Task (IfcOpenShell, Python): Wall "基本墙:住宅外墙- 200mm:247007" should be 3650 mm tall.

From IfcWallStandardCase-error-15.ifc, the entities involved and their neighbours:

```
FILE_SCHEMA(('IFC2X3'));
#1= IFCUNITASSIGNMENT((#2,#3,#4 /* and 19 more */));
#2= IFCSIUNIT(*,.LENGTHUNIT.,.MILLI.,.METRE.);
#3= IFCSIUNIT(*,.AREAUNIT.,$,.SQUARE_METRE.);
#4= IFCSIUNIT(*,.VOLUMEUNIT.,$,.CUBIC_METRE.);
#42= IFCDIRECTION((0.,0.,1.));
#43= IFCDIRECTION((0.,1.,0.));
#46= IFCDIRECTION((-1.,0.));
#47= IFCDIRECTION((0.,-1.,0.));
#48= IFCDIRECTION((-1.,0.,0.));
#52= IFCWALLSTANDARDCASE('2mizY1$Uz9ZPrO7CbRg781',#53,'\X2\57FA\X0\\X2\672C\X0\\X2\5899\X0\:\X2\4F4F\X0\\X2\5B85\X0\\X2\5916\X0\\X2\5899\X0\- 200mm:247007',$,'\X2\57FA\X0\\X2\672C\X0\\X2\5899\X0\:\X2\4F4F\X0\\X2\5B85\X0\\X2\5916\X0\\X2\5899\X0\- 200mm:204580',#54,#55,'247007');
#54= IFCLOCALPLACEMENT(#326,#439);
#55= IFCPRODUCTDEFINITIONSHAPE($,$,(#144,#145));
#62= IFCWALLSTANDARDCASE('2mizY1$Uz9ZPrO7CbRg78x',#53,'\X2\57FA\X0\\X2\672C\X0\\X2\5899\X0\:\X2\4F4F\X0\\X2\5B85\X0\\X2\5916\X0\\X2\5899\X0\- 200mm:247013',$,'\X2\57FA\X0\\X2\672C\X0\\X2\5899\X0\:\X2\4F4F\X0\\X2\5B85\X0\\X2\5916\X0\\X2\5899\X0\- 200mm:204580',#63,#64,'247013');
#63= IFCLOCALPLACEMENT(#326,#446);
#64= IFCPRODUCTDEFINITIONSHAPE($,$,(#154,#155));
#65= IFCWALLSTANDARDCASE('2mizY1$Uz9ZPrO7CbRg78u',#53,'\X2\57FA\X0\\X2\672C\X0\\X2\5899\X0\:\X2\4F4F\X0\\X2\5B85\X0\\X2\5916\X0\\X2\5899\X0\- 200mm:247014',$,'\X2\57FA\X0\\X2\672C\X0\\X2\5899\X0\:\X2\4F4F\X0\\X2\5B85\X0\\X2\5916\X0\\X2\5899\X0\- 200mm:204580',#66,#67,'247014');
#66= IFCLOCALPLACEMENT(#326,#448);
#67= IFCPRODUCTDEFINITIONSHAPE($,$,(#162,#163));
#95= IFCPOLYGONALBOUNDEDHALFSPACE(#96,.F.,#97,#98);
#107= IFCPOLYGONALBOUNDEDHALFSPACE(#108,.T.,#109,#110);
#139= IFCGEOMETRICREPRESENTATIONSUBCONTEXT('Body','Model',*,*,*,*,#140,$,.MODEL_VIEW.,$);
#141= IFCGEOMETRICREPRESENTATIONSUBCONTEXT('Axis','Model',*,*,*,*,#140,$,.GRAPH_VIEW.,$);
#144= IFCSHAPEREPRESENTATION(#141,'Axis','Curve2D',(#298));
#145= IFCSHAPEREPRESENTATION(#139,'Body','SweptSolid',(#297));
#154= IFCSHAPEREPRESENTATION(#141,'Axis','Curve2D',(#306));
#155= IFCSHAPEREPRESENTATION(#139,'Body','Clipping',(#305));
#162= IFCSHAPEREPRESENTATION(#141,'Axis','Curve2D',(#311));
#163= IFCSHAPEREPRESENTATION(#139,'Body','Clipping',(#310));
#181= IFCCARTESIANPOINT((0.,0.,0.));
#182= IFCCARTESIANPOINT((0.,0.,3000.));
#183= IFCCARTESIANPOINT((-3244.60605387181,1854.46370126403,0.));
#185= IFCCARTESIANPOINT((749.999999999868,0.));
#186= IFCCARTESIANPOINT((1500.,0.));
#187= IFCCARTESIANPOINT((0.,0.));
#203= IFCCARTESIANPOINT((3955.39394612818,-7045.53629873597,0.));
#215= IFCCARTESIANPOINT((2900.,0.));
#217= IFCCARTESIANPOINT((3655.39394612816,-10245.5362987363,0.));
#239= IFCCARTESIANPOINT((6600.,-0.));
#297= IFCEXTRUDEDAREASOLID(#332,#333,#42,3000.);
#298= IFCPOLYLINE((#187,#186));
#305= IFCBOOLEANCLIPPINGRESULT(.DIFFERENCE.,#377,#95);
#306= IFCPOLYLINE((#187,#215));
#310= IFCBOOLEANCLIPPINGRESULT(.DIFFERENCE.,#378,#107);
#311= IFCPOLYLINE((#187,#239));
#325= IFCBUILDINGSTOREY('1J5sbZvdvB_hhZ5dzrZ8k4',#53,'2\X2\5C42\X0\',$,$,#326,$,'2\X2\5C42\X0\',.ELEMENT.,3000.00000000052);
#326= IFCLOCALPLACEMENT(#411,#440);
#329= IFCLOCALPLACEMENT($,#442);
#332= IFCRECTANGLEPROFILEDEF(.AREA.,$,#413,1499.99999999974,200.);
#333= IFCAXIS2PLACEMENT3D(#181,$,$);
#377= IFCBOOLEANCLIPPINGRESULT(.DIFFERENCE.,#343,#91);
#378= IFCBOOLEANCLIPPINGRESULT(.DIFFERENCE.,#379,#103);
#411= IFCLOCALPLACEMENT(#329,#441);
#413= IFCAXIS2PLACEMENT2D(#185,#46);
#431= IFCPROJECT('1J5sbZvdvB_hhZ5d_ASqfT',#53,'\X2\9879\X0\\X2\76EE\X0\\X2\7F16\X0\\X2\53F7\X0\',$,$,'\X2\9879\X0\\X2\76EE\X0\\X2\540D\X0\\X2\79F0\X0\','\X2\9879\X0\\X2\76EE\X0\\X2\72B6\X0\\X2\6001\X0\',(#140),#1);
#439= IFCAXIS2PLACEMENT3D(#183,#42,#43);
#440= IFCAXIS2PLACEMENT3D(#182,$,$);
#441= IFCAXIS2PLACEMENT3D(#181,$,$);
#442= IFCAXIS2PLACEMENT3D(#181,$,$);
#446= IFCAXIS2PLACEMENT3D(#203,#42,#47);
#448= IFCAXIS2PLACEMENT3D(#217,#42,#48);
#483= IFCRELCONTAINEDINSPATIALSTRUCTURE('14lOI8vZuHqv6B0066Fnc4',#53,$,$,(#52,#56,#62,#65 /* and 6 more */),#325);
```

```python
import ifcopenshell
import ifcopenshell.geom
import ifcopenshell.util.representation
import ifcopenshell.util.shape

model = ifcopenshell.open("IfcWallStandardCase-error-15.ifc")
settings = ifcopenshell.geom.settings()


def volume(element):
    """Net volume in cubic metres, openings subtracted."""
    shape = ifcopenshell.geom.create_shape(settings, element)
    return ifcopenshell.util.shape.get_volume(shape.geometry)


wall = model.by_guid("2mizY1$Uz9ZPrO7CbRg781")
before = volume(wall)

body = ifcopenshell.util.representation.get_representation(wall, "Model", "Body")
solid = body.Items[0]
old_height = solid.Depth
solid.Depth = 3650.0
after = volume(wall)

print(f"height {old_height:g} -> {solid.Depth:g}, volume {before:.3f} -> {after:.3f} m3")

model.write("IfcWallStandardCase-error-15-out.ifc")
```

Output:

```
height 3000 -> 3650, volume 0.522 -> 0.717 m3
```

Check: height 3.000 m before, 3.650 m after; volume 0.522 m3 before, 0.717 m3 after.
